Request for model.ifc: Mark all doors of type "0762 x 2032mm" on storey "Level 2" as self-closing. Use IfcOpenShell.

First a look at what the model holds.

```python
import ifcopenshell
import ifcopenshell.util.element

model = ifcopenshell.open("model.ifc")
print(model.schema)
storey = next(s for s in model.by_type("IfcBuildingStorey") if s.Name == "Level 2")
doors = [e for e in ifcopenshell.util.element.get_decomposition(storey) if e.is_a("IfcDoor")]
seen = {}
for e in doors:
    element_type = ifcopenshell.util.element.get_type(e)
    key = (element_type.Name if element_type != e and element_type else None, ifcopenshell.util.element.get_pset(e, "Pset_DoorCommon", "SelfClosing"))
    seen[key] = seen.get(key, 0) + 1
for (name, value), count in sorted(seen.items(), key=str):
    print(count, "x", name, "|", value)
```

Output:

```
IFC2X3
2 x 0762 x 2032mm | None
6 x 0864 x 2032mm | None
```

```python
import ifcopenshell
import ifcopenshell.api.pset
import ifcopenshell.util.element

model = ifcopenshell.open("model.ifc")

storey = next(s for s in model.by_type("IfcBuildingStorey") if s.Name == "Level 2")
doors = [e for e in ifcopenshell.util.element.get_decomposition(storey) if e.is_a("IfcDoor")]

count = 0
for e in doors:
    element_type = ifcopenshell.util.element.get_type(e)
    if element_type in (None, e) or element_type.Name != "0762 x 2032mm":
        continue
    # add_pset returns the element's existing set when there is one.
    pset = ifcopenshell.api.pset.add_pset(model, product=e, name="Pset_DoorCommon")
    ifcopenshell.api.pset.edit_pset(model, pset=pset, properties={"SelfClosing": True})
    count += 1

print(count, "doors updated")

model.write("model-out.ifc")
```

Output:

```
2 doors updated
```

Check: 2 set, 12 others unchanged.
